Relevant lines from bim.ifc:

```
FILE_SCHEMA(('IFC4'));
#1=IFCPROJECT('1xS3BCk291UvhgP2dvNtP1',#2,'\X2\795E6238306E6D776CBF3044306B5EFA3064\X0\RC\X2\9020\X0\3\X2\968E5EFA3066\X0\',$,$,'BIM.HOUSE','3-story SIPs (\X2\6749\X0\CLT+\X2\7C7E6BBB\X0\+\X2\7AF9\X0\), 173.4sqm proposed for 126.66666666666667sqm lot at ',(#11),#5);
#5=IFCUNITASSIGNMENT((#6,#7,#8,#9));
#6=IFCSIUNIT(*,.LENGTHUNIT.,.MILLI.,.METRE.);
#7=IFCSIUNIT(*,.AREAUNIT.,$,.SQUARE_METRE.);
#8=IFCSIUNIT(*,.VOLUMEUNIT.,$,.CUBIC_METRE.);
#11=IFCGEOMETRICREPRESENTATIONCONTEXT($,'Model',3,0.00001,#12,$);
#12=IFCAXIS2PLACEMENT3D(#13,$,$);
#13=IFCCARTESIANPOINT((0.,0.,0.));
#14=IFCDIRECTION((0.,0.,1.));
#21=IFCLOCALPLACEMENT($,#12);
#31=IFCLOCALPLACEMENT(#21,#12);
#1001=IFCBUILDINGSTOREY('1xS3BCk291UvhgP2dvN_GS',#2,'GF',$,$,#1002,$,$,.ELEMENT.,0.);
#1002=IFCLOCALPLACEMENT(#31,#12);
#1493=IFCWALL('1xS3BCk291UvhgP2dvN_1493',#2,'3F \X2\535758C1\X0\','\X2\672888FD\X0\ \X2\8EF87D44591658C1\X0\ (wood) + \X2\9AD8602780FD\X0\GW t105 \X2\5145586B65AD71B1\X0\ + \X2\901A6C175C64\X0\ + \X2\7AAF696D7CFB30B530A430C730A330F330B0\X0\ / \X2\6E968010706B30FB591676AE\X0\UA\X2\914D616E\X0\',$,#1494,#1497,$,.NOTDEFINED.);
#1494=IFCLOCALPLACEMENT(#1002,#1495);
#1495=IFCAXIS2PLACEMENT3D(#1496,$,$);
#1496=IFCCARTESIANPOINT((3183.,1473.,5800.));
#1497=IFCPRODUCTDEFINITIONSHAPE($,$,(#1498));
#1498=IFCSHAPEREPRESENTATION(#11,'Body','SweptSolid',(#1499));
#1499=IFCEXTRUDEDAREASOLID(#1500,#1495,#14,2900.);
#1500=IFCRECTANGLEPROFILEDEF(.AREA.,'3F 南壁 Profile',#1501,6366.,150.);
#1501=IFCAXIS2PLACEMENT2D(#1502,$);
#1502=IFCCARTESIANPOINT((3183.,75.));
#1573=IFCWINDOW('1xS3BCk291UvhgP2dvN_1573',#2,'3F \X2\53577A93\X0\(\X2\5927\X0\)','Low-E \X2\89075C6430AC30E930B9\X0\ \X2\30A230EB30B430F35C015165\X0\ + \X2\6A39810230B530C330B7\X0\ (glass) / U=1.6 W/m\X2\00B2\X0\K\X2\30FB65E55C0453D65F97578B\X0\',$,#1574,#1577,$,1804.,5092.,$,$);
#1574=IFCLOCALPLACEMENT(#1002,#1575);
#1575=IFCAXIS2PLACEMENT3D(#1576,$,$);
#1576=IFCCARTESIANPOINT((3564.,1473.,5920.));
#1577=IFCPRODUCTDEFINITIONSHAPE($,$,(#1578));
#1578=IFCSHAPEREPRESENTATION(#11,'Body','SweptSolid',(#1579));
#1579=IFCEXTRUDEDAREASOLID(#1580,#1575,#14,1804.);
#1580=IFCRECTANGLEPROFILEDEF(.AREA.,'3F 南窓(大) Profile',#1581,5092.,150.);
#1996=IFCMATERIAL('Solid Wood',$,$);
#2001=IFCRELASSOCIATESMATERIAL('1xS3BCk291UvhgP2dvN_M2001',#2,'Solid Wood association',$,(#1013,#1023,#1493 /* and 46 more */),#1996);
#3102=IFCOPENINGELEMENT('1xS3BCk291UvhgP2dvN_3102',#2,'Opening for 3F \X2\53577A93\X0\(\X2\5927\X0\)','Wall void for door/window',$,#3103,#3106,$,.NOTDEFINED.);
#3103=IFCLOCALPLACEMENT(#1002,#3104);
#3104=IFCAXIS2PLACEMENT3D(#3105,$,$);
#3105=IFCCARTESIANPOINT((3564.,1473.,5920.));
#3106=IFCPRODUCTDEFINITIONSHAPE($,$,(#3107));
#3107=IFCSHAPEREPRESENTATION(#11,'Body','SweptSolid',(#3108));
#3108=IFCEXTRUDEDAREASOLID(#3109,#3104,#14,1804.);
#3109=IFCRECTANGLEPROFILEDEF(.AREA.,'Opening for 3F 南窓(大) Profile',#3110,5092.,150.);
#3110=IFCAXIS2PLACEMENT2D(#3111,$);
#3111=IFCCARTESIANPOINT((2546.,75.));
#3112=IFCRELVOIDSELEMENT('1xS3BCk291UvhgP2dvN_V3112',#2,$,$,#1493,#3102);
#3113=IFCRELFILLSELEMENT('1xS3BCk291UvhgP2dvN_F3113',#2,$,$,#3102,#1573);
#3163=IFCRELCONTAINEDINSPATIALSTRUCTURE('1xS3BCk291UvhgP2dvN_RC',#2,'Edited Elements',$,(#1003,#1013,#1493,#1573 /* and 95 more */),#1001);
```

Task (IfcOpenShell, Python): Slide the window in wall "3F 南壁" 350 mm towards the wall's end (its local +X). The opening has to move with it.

```python
import ifcopenshell
import ifcopenshell.api.geometry
import ifcopenshell.util.placement

model = ifcopenshell.open("bim.ifc")

window = model.by_guid("1xS3BCk291UvhgP2dvN_1573")
opening = window.FillsVoids[0].RelatingOpeningElement
wall = opening.VoidsElements[0].RelatingBuildingElement

wall_matrix = ifcopenshell.util.placement.get_local_placement(wall.ObjectPlacement)
shift = wall_matrix[:3, 0] * 350.0
before = ifcopenshell.util.placement.get_local_placement(window.ObjectPlacement)[:3, 3].copy()

# The window is not placed relative to its opening, so move both.
for product in (opening, window):
    matrix = ifcopenshell.util.placement.get_local_placement(product.ObjectPlacement)
    matrix[:3, 3] += shift
    ifcopenshell.api.geometry.edit_object_placement(model, product=product, matrix=matrix, is_si=False)

after = ifcopenshell.util.placement.get_local_placement(window.ObjectPlacement)[:3, 3]
print("window moved by", (after - before).round(3) + 0.0)

model.write("bim_edited.ifc")
```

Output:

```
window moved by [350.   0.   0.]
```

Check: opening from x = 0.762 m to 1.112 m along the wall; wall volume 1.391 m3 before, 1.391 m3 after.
